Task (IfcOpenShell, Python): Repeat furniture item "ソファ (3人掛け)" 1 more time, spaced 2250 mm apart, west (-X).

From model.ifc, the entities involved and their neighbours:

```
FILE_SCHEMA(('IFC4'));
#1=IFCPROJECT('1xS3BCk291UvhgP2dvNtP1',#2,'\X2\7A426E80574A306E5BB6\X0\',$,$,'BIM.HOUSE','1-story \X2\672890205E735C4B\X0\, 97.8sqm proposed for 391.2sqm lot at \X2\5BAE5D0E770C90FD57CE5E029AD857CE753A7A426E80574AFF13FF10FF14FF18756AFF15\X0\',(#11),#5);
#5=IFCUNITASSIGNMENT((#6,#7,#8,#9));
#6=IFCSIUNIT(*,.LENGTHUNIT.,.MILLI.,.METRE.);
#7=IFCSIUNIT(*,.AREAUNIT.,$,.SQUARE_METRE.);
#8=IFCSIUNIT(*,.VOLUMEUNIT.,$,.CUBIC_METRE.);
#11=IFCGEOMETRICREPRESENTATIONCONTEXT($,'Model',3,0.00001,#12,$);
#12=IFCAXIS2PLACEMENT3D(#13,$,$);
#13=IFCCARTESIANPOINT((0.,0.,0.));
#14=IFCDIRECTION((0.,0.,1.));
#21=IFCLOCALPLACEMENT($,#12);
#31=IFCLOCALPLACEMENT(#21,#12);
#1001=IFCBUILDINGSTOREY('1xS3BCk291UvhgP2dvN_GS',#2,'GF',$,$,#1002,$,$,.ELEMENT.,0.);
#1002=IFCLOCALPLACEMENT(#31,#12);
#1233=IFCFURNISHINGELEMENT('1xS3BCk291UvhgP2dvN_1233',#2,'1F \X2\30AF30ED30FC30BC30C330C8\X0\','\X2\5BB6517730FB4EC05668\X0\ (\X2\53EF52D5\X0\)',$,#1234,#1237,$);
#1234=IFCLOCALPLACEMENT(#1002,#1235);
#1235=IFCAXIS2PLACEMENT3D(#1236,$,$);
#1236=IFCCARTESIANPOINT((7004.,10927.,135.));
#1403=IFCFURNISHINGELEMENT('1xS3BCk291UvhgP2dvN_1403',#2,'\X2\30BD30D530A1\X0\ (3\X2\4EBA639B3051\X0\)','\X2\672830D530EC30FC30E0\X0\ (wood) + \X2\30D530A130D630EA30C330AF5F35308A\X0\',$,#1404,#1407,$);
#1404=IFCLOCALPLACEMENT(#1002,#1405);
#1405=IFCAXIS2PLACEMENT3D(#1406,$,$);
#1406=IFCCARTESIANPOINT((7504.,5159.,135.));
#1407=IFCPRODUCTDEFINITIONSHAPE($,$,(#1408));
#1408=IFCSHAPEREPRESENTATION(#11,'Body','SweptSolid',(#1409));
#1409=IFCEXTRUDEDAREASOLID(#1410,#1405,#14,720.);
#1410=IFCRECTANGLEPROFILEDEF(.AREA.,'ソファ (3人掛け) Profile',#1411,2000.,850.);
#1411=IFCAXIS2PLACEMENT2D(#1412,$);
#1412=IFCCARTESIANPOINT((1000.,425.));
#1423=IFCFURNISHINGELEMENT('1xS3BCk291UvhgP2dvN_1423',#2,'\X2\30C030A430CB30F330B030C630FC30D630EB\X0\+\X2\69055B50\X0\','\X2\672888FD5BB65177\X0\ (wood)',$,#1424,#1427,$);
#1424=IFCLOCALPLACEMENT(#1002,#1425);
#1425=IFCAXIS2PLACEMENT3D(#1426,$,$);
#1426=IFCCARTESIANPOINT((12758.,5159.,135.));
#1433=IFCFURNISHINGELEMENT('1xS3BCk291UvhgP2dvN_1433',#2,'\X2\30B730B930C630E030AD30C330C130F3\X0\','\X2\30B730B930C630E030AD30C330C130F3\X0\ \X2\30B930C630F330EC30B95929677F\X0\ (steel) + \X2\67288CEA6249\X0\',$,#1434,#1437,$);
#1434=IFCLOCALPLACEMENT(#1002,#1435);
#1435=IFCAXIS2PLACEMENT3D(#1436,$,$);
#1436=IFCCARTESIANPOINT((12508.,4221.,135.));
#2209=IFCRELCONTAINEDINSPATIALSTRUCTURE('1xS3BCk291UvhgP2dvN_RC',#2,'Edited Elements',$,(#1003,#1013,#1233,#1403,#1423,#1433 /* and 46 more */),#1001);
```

```python
import numpy as np
import ifcopenshell
import ifcopenshell.api.geometry
import ifcopenshell.api.root
import ifcopenshell.util.element
import ifcopenshell.util.placement
import ifcopenshell.util.unit

model = ifcopenshell.open("model.ifc")
unit_scale = ifcopenshell.util.unit.calculate_unit_scale(model)


def reuse_history(source, copy):
    """copy_class also copies each property set's owner history, people and application; keep the originals."""
    for rel in copy.IsDefinedBy:
        if rel.is_a("IfcRelDefinesByProperties") and (history := rel.RelatingPropertyDefinition.OwnerHistory):
            rel.RelatingPropertyDefinition.OwnerHistory = source.OwnerHistory
            ifcopenshell.util.element.remove_deep2(model, history)


source = model.by_guid("1xS3BCk291UvhgP2dvN_1403")
base = ifcopenshell.util.placement.get_local_placement(source.ObjectPlacement)
step = np.array([-1.0, 0.0, 0.0]) * 2.25 / unit_scale

for i in range(1, 2):
    copy = ifcopenshell.api.root.copy_class(model, product=source)
    copy.Representation = ifcopenshell.util.element.copy_deep(
        model, source.Representation, exclude=["IfcGeometricRepresentationContext", "IfcRepresentationMap"]
    )
    reuse_history(source, copy)
    matrix = base.copy()
    matrix[:3, 3] += i * step
    print("added at", matrix[:3, 3].round(3) + 0.0)
    ifcopenshell.api.geometry.edit_object_placement(model, product=copy, matrix=matrix, is_si=False)

model.write("model-out.ifc")
```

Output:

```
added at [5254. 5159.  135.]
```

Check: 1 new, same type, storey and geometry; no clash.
